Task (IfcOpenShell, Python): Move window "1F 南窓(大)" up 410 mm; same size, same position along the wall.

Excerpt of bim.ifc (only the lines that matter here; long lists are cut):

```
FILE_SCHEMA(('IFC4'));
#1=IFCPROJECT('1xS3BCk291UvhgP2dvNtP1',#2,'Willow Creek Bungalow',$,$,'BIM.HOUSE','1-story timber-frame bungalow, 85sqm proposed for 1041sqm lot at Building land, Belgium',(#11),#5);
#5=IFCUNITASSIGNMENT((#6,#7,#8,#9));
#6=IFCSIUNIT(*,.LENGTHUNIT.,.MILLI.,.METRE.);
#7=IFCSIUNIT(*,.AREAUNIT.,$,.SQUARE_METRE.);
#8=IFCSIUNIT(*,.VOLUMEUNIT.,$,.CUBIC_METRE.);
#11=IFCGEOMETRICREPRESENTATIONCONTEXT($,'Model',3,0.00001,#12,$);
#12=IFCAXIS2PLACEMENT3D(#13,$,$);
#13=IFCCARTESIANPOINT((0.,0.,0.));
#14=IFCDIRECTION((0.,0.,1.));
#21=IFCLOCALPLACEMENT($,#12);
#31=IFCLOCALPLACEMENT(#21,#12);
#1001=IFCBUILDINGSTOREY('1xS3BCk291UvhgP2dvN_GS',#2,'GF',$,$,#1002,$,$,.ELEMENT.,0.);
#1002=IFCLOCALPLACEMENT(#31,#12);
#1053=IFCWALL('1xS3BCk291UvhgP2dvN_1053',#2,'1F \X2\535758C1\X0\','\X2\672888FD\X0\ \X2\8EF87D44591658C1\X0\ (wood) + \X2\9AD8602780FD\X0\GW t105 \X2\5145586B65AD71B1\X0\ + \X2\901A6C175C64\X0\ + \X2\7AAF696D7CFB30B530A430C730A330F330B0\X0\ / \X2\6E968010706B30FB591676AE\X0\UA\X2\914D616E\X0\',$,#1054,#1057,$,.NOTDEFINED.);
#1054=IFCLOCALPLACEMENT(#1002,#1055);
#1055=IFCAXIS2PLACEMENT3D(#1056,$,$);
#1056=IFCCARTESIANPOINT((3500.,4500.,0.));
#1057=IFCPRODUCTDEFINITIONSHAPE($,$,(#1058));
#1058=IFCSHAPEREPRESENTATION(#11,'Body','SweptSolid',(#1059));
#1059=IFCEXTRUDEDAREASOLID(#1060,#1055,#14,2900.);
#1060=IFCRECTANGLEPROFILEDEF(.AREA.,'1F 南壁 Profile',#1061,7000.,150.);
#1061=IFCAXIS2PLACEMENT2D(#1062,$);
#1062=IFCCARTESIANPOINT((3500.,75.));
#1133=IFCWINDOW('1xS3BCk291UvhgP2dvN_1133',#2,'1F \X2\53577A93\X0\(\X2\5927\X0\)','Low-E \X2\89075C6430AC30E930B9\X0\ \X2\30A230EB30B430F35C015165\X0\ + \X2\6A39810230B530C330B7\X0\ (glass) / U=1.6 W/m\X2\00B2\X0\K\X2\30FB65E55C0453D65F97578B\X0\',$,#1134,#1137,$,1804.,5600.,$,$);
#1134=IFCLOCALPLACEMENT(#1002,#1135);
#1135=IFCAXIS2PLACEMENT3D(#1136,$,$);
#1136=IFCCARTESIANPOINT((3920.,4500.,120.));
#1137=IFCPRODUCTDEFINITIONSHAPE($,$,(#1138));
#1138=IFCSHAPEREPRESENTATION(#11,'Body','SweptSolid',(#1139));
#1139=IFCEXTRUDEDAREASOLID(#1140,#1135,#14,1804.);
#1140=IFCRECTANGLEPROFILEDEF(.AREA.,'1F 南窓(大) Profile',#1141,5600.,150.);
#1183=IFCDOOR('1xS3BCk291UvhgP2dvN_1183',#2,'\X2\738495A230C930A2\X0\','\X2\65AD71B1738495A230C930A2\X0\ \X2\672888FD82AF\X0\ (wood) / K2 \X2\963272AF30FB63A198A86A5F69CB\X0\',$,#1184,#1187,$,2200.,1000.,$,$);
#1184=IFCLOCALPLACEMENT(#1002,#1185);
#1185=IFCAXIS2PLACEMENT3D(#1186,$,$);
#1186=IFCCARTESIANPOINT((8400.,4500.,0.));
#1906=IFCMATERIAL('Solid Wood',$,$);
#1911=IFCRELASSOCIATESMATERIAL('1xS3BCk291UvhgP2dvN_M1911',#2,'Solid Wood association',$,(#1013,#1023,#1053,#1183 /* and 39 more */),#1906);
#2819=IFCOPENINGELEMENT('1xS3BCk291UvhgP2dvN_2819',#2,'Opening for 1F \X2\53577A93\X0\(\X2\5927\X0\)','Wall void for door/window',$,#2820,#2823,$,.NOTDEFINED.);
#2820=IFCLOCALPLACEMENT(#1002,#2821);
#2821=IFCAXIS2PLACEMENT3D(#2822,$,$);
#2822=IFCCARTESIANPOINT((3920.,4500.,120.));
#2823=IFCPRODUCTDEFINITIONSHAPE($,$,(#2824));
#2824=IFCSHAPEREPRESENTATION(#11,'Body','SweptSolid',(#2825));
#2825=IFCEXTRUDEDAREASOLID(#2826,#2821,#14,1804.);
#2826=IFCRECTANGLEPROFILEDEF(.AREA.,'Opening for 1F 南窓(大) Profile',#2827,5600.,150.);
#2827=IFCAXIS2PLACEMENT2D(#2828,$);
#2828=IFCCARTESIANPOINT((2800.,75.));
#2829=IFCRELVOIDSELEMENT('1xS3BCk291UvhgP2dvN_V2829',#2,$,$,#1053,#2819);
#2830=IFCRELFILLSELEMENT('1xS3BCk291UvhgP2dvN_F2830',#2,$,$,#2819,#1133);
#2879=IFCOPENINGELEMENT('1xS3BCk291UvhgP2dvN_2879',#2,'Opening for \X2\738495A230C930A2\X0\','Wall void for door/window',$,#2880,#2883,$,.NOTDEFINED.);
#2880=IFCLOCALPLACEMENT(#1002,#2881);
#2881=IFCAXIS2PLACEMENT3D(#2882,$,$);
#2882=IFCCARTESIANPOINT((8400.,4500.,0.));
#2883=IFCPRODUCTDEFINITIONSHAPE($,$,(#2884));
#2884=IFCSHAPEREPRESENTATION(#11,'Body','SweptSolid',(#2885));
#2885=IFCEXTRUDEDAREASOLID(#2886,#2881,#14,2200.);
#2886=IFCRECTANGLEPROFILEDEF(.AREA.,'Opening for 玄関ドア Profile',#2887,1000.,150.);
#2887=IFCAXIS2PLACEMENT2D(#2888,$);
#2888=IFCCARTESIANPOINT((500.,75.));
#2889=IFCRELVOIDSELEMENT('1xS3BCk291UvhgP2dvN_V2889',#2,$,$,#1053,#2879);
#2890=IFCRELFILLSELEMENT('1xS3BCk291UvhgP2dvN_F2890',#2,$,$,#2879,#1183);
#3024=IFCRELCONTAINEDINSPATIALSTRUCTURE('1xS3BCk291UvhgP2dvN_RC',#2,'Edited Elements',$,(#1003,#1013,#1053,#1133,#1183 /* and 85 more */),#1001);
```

```python
import numpy as np
import ifcopenshell
import ifcopenshell.api.geometry
import ifcopenshell.util.placement
import ifcopenshell.util.unit

model = ifcopenshell.open("bim.ifc")
unit_scale = ifcopenshell.util.unit.calculate_unit_scale(model)

window = model.by_guid("1xS3BCk291UvhgP2dvN_1133")
opening = window.FillsVoids[0].RelatingOpeningElement
dz = 0.41 / unit_scale

shift = np.array([0.0, 0.0, dz])
# The window is not placed relative to its opening, so move both.
for product in (opening, window):
    matrix = ifcopenshell.util.placement.get_local_placement(product.ObjectPlacement)
    matrix[:3, 3] += shift
    ifcopenshell.api.geometry.edit_object_placement(model, product=product, matrix=matrix, is_si=False)

print(f"moved by {dz * unit_scale:+.3f} m")

model.write("bim_updated.ifc")
```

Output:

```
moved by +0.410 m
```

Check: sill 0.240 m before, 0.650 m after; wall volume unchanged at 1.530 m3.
